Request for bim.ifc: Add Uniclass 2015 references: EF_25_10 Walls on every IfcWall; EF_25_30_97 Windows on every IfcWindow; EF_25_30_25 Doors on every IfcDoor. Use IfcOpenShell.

First a look at what the model holds.

```python
import ifcopenshell

model = ifcopenshell.open("bim.ifc")
print(model.schema)
print("classifications:", [c.Name for c in model.by_type("IfcClassification")])
for ifc_class in ("IfcDoor", "IfcRoof", "IfcStair", "IfcWall", "IfcWindow"):
    print(ifc_class, len(model.by_type(ifc_class)))
```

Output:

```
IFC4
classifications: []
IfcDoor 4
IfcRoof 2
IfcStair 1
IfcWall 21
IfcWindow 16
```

```python
import ifcopenshell
import ifcopenshell.api.classification

model = ifcopenshell.open("bim.ifc")

system = ifcopenshell.api.classification.add_classification(model, classification="Uniclass 2015")

codes = {
    "IfcWall": ("EF_25_10", "Walls"),
    "IfcWindow": ("EF_25_30_97", "Windows"),
    "IfcDoor": ("EF_25_30_25", "Doors"),
}
for ifc_class, (code, name) in codes.items():
    products = model.by_type(ifc_class)
    ifcopenshell.api.classification.add_reference(
        model, products=products, classification=system, identification=code, name=name
    )
    print(code, len(products))

model.write("bim_v2.ifc")
```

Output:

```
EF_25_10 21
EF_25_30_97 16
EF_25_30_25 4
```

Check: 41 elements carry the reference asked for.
